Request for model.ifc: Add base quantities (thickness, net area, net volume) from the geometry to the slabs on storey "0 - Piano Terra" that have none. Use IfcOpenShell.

First a look at what the model holds.

```python
import ifcopenshell
import ifcopenshell.util.element
import ifcopenshell.util.unit

model = ifcopenshell.open("model.ifc")
print(model.schema)
for unit_type in ("LENGTHUNIT", "AREAUNIT", "VOLUMEUNIT"):
    print(unit_type, ifcopenshell.util.unit.calculate_unit_scale(model, unit_type))
storey = next(s for s in model.by_type("IfcBuildingStorey") if s.Name == "0 - Piano Terra")
slabs = [e for e in ifcopenshell.util.element.get_decomposition(storey) if e.is_a("IfcSlab")]
for e in sorted(slabs, key=lambda e: e.id()):
    print(e.id(), e.is_a(), e.Name, list(ifcopenshell.util.element.get_psets(e, qtos_only=True)), sep=" | ")
```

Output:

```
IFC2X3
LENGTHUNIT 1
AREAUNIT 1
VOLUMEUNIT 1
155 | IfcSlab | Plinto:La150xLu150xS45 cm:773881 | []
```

```python
import ifcopenshell
import ifcopenshell.api.pset
import ifcopenshell.geom
import ifcopenshell.util.element
import ifcopenshell.util.shape
import ifcopenshell.util.unit

model = ifcopenshell.open("model.ifc")
unit_scale = ifcopenshell.util.unit.calculate_unit_scale(model)
area_scale = ifcopenshell.util.unit.calculate_unit_scale(model, "AREAUNIT")
volume_scale = ifcopenshell.util.unit.calculate_unit_scale(model, "VOLUMEUNIT")
settings = ifcopenshell.geom.settings()

storey = next(s for s in model.by_type("IfcBuildingStorey") if s.Name == "0 - Piano Terra")
slabs = [e for e in ifcopenshell.util.element.get_decomposition(storey) if e.is_a("IfcSlab")]

for e in sorted(slabs, key=lambda e: e.id()):
    if ifcopenshell.util.element.get_psets(e, qtos_only=True, should_inherit=False):
        continue
    # Geometry comes back in metres, in the element's own axes.
    shape = ifcopenshell.geom.create_shape(settings, e)
    values = {
        "Width": ifcopenshell.util.shape.get_z(shape.geometry) / unit_scale,
        "NetArea": ifcopenshell.util.shape.get_footprint_area(shape.geometry) / area_scale,
        "NetVolume": ifcopenshell.util.shape.get_volume(shape.geometry) / volume_scale,
    }
    qto = ifcopenshell.api.pset.add_qto(model, product=e, name="BaseQuantities")
    ifcopenshell.api.pset.edit_qto(model, qto=qto, properties=values)
    print(e.id(), {k: round(v, 3) for k, v in values.items()})

model.write("model_updated.ifc")
```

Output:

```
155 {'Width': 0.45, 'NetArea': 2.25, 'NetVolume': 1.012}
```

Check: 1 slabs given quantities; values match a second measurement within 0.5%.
